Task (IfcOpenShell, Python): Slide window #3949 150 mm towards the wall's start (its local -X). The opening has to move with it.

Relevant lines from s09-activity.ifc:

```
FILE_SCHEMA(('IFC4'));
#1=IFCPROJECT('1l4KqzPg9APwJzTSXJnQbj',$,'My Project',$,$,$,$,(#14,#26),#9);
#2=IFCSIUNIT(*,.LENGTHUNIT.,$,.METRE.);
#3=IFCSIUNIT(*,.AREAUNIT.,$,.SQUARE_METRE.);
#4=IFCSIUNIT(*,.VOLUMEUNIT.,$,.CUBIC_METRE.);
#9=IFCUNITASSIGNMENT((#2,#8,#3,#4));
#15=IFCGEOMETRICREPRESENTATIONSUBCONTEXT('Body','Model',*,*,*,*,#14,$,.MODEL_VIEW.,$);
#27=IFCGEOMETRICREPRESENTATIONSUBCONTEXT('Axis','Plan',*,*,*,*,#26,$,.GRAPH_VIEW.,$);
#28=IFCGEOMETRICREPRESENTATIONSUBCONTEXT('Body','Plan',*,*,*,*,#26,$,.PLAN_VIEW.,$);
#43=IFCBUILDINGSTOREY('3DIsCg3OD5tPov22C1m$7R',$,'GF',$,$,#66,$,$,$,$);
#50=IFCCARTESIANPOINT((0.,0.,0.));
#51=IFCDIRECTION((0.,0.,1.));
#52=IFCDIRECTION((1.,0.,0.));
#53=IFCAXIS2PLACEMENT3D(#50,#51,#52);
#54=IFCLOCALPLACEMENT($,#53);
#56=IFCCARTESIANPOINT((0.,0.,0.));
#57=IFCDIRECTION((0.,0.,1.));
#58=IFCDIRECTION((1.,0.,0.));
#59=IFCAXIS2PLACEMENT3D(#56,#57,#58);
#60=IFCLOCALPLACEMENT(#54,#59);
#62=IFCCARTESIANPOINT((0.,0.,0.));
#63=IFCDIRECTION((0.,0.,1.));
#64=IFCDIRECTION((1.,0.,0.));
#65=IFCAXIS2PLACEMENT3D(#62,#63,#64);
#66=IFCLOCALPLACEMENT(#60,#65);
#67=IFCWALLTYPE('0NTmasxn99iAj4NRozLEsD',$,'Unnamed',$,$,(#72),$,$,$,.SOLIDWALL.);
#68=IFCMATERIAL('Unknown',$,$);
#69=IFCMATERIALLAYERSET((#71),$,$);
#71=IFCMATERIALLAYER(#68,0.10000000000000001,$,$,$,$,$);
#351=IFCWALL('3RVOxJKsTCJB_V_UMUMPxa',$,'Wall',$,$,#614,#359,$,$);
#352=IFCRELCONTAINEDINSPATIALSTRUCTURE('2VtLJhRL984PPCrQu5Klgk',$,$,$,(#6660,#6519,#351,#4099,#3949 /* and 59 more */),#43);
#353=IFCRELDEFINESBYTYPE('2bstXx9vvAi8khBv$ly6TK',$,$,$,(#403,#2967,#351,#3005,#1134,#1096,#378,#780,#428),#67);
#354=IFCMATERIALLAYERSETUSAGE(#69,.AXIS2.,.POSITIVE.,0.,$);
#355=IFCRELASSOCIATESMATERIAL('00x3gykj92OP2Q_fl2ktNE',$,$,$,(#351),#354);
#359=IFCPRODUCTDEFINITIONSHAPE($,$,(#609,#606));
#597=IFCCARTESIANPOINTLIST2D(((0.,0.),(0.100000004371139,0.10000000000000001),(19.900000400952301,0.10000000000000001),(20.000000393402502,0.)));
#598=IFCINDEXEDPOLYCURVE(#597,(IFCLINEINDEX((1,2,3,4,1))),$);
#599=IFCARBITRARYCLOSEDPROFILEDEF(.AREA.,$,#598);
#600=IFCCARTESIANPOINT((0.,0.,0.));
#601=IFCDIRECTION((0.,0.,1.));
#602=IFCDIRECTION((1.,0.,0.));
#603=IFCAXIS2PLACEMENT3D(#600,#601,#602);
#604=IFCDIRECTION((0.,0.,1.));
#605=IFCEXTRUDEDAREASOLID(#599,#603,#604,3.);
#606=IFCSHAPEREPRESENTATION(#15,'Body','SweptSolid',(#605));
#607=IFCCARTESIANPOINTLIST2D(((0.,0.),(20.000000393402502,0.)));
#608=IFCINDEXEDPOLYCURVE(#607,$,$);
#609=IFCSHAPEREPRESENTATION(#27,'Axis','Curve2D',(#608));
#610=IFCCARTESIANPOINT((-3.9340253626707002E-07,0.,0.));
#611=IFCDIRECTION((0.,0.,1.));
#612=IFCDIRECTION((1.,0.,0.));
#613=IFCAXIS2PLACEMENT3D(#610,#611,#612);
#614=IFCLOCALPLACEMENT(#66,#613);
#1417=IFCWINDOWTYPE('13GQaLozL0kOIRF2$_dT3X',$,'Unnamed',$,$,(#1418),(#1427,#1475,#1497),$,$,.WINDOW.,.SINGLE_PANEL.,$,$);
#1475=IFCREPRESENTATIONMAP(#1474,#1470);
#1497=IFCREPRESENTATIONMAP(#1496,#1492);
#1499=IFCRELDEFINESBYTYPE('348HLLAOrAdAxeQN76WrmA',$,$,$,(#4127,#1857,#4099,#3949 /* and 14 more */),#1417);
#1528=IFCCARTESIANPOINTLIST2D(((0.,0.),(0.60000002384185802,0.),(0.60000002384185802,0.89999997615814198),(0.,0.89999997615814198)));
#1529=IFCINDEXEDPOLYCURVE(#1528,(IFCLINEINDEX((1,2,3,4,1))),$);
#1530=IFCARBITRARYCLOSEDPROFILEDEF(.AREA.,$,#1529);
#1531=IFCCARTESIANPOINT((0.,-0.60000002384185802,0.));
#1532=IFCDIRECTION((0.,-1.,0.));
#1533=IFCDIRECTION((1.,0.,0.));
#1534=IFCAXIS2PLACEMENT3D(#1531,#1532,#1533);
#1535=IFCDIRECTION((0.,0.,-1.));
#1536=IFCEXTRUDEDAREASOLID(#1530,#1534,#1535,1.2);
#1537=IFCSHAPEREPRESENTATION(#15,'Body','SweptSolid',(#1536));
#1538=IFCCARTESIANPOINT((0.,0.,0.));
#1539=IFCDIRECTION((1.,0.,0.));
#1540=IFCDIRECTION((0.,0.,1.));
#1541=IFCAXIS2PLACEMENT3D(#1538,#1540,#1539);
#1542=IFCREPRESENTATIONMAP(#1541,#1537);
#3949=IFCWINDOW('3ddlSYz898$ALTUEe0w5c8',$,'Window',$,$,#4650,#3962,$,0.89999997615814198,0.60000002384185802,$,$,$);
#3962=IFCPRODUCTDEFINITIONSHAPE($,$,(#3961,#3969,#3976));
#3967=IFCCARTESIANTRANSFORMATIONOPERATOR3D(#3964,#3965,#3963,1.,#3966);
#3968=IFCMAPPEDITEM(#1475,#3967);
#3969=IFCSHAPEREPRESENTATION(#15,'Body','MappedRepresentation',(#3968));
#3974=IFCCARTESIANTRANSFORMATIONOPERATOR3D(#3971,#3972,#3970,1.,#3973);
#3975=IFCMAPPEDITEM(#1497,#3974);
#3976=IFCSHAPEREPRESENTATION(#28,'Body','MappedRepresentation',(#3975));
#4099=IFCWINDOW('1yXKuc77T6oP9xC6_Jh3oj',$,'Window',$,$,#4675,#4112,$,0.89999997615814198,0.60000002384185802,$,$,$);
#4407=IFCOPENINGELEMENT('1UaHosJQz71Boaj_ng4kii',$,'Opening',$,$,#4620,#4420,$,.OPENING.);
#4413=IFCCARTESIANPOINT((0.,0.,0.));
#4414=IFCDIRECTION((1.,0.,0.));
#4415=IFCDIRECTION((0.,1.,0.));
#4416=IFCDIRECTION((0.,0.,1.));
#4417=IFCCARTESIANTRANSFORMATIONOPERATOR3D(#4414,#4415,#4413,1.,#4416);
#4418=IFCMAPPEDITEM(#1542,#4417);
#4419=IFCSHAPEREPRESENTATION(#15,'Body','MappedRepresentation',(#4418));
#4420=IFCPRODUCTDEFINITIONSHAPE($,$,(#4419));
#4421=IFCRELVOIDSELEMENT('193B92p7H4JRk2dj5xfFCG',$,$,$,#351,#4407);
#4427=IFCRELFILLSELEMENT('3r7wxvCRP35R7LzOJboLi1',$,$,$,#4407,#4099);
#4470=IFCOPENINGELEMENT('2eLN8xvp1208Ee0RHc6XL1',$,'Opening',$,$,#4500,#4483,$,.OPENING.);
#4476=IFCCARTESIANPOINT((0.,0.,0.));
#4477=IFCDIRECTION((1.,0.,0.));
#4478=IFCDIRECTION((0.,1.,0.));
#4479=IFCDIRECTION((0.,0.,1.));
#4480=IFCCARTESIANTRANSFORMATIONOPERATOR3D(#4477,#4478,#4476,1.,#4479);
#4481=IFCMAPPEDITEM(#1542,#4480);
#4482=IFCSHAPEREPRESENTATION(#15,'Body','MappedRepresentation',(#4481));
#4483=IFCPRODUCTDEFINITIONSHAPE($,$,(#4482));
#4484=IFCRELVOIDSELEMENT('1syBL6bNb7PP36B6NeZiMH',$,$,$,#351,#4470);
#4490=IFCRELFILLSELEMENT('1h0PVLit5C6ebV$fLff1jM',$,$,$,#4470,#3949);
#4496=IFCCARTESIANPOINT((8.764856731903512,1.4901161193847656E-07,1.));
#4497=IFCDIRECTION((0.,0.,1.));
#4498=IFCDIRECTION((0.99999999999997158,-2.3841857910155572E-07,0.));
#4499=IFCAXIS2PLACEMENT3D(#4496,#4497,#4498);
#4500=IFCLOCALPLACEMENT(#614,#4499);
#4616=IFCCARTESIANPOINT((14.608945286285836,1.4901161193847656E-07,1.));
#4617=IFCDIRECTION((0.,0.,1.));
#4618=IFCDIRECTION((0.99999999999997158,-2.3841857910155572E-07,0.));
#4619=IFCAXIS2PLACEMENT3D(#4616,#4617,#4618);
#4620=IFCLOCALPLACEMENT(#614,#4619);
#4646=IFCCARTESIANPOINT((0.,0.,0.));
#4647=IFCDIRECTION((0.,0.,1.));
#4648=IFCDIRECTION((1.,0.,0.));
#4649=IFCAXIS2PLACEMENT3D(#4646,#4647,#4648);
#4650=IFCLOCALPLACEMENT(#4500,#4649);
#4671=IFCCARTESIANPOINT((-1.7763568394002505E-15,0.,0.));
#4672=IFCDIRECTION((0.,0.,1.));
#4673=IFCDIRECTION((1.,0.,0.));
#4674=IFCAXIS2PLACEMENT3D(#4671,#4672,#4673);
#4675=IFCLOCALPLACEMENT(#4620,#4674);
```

```python
import ifcopenshell
import ifcopenshell.api.geometry
import ifcopenshell.util.placement
import ifcopenshell.util.unit

model = ifcopenshell.open("s09-activity.ifc")
unit_scale = ifcopenshell.util.unit.calculate_unit_scale(model)

window = model.by_guid("3ddlSYz898$ALTUEe0w5c8")
opening = window.FillsVoids[0].RelatingOpeningElement
wall = opening.VoidsElements[0].RelatingBuildingElement

wall_matrix = ifcopenshell.util.placement.get_local_placement(wall.ObjectPlacement)
shift = wall_matrix[:3, 0] * -0.15 / unit_scale
before = ifcopenshell.util.placement.get_local_placement(window.ObjectPlacement)[:3, 3].copy()

# The window is placed relative to its opening, so it follows when the opening moves.
matrix = ifcopenshell.util.placement.get_local_placement(opening.ObjectPlacement)
matrix[:3, 3] += shift
ifcopenshell.api.geometry.edit_object_placement(
    model, product=opening, matrix=matrix, is_si=False, should_transform_children=True
)

after = ifcopenshell.util.placement.get_local_placement(window.ObjectPlacement)[:3, 3]
print("window moved by", (after - before).round(3) + 0.0)

model.write("s09-activity_updated.ifc")
```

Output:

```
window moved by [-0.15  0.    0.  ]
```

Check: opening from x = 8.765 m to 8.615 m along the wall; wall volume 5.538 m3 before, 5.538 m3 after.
